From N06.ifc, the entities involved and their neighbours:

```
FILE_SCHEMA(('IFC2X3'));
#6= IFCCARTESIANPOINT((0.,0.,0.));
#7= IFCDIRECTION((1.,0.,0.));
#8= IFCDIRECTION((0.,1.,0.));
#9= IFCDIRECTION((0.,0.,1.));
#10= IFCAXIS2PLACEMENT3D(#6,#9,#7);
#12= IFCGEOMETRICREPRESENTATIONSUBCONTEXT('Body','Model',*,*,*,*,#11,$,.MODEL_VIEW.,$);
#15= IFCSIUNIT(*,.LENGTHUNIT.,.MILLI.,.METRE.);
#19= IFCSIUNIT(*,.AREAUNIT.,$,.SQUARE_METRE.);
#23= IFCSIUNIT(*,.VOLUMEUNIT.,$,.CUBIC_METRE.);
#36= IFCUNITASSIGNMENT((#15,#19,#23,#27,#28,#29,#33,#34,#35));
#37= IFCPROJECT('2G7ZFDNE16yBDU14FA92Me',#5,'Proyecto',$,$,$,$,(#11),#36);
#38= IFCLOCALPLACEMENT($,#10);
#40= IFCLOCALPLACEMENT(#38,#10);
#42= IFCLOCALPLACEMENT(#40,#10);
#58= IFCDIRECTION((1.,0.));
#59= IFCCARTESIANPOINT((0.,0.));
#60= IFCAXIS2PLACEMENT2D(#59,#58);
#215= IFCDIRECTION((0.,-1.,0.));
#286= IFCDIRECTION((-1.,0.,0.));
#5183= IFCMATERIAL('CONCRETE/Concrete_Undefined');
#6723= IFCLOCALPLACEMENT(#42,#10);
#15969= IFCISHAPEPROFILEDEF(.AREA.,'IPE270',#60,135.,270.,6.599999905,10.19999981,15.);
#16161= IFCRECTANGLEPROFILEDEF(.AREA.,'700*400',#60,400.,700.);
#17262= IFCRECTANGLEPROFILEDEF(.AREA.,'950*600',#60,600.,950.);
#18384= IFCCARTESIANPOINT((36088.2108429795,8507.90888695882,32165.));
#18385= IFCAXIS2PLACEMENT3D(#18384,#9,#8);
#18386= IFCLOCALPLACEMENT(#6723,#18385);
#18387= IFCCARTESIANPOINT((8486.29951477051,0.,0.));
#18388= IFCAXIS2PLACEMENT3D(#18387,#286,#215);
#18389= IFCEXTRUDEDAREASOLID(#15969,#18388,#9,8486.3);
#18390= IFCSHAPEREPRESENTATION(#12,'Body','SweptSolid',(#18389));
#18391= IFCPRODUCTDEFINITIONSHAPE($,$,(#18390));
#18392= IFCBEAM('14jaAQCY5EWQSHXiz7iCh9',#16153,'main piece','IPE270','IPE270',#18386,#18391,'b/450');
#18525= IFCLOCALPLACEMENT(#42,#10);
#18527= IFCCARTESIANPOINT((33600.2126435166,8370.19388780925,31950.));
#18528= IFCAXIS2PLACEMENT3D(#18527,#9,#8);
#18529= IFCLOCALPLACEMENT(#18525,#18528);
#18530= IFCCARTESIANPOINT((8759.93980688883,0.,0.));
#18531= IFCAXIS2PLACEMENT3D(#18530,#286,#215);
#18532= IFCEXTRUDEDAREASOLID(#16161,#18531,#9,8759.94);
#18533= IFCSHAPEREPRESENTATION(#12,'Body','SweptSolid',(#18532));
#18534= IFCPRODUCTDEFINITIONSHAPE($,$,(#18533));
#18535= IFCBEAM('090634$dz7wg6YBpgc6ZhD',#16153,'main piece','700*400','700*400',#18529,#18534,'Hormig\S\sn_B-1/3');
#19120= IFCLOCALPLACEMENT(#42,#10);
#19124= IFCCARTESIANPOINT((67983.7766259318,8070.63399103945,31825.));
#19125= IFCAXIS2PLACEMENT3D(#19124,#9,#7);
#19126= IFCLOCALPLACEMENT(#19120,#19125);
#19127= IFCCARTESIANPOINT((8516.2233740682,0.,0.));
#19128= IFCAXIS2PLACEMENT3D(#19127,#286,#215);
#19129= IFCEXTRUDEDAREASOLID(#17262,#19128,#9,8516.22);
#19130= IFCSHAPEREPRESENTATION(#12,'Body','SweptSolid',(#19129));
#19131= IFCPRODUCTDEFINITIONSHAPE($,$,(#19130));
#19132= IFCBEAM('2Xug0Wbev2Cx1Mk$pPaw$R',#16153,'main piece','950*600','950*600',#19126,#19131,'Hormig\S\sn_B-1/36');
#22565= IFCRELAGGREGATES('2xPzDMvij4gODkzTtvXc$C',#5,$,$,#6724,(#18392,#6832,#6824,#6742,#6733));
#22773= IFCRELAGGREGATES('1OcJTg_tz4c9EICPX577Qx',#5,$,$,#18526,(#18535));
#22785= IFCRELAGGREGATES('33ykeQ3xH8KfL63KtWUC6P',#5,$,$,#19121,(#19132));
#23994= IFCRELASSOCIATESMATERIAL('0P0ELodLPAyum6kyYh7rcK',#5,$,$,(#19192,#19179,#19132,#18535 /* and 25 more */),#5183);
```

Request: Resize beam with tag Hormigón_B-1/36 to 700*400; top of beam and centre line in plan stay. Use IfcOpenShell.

```python
import ifcopenshell
import ifcopenshell.util.element
import ifcopenshell.util.representation

model = ifcopenshell.open("N06.ifc")

member = model.by_guid("2Xug0Wbev2Cx1Mk$pPaw$R")
source = next(p for p in model.by_type("IfcRectangleProfileDef") if p.ProfileName == "700*400")

body = ifcopenshell.util.representation.get_representation(member, "Model", "Body")
solid = body.Items[0]
old_profile = solid.SweptArea

# Copy the section's sizes but keep this member's own profile position.
profile = ifcopenshell.util.element.copy(model, source)
# Profiles are centred, so shift by half the change in depth to hold the top.
shift = (old_profile.YDim - profile.YDim) / 2
x, y = old_profile.Position.Location.Coordinates
up = (0.0, 1.0)  # upwards, in the solid's own plane
location = model.createIfcCartesianPoint((x + up[0] * shift, y + up[1] * shift))
profile.Position = model.createIfcAxis2Placement2D(location, old_profile.Position.RefDirection)
solid.SweptArea = profile
if not model.get_total_inverses(old_profile):
    ifcopenshell.util.element.remove_deep2(model, old_profile)
member.Description = member.Description.replace("950*600", "700*400")
member.ObjectType = member.ObjectType.replace("950*600", "700*400")

print(solid.SweptArea)

model.write("N06_edited.ifc")
```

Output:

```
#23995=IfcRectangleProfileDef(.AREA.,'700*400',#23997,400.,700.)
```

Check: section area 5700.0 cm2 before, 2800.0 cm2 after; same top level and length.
